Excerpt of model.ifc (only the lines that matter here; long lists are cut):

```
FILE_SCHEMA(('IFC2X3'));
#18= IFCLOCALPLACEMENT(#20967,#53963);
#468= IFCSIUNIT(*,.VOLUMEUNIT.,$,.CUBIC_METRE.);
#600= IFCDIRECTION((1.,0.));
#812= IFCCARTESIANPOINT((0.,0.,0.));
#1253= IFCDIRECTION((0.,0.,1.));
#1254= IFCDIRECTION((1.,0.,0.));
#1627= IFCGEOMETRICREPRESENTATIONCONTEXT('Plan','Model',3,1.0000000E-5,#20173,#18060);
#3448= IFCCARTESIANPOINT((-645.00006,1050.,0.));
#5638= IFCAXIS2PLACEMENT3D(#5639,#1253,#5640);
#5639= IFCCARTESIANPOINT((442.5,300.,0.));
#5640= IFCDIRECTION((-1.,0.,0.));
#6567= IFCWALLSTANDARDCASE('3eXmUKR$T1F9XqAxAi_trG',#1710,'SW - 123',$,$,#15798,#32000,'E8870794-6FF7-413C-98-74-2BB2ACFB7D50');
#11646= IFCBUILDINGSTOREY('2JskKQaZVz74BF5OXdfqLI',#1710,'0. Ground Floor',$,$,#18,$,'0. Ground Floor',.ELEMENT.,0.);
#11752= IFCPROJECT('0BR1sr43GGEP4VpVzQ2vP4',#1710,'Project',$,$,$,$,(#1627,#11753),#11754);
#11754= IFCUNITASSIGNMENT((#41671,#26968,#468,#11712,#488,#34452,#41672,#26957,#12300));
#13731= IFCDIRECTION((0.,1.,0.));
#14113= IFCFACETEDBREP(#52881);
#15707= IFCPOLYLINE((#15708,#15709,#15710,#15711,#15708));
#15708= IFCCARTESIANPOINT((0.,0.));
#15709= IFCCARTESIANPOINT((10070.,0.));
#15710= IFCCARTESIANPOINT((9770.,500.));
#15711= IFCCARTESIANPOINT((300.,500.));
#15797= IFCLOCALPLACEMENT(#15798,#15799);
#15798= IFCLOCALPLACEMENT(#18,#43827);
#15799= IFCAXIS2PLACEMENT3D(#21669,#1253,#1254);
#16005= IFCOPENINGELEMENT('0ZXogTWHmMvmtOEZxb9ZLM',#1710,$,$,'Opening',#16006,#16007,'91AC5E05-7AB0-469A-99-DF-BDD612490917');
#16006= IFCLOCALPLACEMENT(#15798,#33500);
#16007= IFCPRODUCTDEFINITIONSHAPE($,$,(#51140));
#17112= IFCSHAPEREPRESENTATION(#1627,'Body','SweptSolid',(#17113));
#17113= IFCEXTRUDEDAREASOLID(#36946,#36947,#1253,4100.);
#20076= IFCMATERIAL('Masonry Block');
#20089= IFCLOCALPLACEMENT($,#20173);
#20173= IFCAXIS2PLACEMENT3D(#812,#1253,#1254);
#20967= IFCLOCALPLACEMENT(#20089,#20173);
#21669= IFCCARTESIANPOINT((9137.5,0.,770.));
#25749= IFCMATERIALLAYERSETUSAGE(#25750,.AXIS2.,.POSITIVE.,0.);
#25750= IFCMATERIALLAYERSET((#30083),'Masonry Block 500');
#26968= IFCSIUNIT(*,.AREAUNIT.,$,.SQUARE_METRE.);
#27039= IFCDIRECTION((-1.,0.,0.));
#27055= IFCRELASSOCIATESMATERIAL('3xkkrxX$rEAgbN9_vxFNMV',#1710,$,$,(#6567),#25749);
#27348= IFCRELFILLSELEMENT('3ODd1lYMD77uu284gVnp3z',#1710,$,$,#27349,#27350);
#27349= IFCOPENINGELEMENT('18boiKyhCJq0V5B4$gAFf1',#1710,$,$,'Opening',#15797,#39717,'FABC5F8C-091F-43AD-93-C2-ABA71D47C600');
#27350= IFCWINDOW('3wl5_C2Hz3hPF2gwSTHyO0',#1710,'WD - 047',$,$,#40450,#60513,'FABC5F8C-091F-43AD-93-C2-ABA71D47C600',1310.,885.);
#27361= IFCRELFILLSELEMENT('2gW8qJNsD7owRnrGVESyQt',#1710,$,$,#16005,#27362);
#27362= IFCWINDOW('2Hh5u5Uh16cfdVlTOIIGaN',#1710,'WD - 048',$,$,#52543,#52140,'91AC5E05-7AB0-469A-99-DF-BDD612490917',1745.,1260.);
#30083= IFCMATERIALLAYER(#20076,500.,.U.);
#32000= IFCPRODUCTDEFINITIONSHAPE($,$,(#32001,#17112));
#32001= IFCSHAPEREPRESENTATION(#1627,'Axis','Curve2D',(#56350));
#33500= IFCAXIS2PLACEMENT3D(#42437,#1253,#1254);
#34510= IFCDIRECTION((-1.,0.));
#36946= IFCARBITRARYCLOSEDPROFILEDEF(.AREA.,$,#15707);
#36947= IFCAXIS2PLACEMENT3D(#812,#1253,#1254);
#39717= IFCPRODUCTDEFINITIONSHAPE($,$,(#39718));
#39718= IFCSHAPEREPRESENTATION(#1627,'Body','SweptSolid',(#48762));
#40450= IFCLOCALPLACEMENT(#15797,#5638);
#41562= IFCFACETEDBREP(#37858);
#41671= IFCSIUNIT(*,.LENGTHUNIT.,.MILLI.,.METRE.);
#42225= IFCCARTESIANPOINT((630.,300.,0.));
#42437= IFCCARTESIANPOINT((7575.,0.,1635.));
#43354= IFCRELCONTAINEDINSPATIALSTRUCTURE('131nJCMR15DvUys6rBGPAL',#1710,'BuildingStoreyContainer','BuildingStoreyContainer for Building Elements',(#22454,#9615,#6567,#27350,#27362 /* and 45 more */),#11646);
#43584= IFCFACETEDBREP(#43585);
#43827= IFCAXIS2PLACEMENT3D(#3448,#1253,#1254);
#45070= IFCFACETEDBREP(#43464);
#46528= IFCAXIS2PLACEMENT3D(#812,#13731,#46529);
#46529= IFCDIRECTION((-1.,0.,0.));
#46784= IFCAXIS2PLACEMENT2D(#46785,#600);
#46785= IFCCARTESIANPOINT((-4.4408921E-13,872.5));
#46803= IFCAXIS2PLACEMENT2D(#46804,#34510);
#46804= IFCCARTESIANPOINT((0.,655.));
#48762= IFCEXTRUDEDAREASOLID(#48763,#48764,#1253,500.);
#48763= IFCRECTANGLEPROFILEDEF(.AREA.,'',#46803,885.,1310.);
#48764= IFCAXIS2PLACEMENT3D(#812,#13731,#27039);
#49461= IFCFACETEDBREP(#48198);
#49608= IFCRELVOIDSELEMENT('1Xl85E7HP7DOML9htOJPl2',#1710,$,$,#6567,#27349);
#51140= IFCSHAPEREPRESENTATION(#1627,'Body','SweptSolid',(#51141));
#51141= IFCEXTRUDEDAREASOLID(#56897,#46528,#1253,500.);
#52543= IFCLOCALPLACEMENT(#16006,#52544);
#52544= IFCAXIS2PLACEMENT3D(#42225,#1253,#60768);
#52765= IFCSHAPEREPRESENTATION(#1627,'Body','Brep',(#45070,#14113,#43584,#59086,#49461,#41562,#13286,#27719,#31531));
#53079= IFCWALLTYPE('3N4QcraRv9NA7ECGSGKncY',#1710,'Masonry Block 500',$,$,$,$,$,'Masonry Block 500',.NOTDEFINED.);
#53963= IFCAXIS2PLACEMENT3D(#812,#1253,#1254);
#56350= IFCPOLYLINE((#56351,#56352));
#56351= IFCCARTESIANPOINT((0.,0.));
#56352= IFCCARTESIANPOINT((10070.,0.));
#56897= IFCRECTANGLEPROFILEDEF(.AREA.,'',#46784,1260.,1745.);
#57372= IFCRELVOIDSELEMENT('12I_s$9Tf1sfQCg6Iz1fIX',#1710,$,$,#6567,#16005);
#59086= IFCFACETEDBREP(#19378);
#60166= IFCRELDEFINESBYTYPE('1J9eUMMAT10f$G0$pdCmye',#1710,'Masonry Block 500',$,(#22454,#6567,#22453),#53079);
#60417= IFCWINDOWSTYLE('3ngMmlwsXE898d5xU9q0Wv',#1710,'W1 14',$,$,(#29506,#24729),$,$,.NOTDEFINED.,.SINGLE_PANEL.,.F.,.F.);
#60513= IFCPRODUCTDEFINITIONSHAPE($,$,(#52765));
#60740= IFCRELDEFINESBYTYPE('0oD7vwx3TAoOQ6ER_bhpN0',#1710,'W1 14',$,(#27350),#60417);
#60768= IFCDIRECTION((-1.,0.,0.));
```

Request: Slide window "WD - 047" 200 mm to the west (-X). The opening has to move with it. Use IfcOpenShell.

```python
import ifcopenshell
import ifcopenshell.api.geometry
import ifcopenshell.util.placement
import ifcopenshell.util.unit

model = ifcopenshell.open("model.ifc")
unit_scale = ifcopenshell.util.unit.calculate_unit_scale(model)

window = model.by_guid("3wl5_C2Hz3hPF2gwSTHyO0")
opening = window.FillsVoids[0].RelatingOpeningElement
wall = opening.VoidsElements[0].RelatingBuildingElement

wall_matrix = ifcopenshell.util.placement.get_local_placement(wall.ObjectPlacement)
shift = wall_matrix[:3, 0] * -0.2 / unit_scale
before = ifcopenshell.util.placement.get_local_placement(window.ObjectPlacement)[:3, 3].copy()

# The window is placed relative to its opening, so it follows when the opening moves.
matrix = ifcopenshell.util.placement.get_local_placement(opening.ObjectPlacement)
matrix[:3, 3] += shift
ifcopenshell.api.geometry.edit_object_placement(
    model, product=opening, matrix=matrix, is_si=False, should_transform_children=True
)

after = ifcopenshell.util.placement.get_local_placement(window.ObjectPlacement)[:3, 3]
print("window moved by", (after - before).round(3) + 0.0)

model.write("model_edited.ifc")
```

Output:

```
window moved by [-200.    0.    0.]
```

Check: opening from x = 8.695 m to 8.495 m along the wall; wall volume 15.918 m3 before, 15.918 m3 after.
